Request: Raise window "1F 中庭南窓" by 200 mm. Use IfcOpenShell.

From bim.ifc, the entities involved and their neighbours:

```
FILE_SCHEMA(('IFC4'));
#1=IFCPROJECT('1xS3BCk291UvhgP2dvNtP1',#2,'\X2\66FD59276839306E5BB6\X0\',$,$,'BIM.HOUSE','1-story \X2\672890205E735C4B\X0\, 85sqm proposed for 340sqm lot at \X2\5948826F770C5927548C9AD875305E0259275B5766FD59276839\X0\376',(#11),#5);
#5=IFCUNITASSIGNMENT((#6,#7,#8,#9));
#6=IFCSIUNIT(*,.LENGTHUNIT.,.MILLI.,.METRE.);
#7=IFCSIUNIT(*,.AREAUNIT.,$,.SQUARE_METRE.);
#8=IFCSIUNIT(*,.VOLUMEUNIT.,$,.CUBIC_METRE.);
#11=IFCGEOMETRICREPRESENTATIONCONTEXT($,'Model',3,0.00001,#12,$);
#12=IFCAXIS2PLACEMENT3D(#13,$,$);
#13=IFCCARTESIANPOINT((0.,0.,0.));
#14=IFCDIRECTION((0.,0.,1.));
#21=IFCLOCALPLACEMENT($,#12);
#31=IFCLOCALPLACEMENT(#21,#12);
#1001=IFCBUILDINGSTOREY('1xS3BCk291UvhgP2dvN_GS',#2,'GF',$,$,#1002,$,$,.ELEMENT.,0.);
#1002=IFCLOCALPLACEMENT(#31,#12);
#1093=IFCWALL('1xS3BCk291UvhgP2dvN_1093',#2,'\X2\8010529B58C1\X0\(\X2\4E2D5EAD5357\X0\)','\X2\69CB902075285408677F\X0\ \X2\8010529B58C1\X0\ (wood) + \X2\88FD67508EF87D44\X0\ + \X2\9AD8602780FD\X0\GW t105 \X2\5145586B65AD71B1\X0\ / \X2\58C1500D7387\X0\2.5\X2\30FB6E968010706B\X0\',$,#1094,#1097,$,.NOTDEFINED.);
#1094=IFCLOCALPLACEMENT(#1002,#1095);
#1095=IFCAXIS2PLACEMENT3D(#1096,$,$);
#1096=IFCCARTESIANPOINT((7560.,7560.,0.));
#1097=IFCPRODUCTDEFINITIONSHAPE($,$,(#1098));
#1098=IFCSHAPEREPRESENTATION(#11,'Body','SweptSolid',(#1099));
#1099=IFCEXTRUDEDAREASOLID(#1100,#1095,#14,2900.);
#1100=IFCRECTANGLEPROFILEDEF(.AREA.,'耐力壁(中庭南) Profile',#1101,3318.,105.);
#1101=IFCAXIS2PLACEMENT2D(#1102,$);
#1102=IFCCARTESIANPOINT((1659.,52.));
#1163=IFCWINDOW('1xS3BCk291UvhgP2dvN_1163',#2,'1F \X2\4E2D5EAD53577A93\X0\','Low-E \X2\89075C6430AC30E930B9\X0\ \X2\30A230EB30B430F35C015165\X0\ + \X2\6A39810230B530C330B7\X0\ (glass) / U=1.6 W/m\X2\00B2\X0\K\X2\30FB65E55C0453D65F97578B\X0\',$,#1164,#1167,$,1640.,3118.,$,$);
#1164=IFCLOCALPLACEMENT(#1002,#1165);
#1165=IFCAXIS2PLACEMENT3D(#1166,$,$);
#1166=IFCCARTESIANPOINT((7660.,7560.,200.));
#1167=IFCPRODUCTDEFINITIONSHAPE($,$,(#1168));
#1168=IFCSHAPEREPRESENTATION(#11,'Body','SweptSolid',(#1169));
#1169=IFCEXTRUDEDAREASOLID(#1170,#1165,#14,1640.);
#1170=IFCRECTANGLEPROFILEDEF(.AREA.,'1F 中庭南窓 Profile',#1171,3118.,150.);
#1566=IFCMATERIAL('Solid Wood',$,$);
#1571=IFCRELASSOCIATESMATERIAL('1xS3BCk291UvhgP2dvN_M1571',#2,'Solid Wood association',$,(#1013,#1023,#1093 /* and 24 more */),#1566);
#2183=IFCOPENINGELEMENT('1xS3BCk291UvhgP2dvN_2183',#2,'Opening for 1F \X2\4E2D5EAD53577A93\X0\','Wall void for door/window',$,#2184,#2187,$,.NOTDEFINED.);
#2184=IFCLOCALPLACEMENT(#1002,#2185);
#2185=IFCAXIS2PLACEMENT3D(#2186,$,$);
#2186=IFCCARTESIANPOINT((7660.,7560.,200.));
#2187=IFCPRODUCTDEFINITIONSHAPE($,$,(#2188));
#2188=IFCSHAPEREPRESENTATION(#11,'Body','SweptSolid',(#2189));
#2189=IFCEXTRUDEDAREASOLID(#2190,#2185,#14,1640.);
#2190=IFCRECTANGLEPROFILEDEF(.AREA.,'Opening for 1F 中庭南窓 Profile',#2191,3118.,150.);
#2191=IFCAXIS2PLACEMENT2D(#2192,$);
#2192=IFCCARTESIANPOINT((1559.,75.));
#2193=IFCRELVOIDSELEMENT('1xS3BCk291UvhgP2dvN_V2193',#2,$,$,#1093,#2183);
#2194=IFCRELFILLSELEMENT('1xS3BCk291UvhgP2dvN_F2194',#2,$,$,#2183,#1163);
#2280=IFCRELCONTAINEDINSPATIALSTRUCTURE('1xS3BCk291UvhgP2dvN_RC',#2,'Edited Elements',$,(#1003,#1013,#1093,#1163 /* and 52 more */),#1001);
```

```python
import numpy as np
import ifcopenshell
import ifcopenshell.api.geometry
import ifcopenshell.util.placement
import ifcopenshell.util.unit

model = ifcopenshell.open("bim.ifc")
unit_scale = ifcopenshell.util.unit.calculate_unit_scale(model)

window = model.by_id(1163)
opening = window.FillsVoids[0].RelatingOpeningElement
dz = 0.2 / unit_scale

shift = np.array([0.0, 0.0, dz])
# The window is not placed relative to its opening, so move both.
for product in (opening, window):
    matrix = ifcopenshell.util.placement.get_local_placement(product.ObjectPlacement)
    matrix[:3, 3] += shift
    ifcopenshell.api.geometry.edit_object_placement(model, product=product, matrix=matrix, is_si=False)

print(f"moved by {dz * unit_scale:+.3f} m")

model.write("bim-out.ifc")
```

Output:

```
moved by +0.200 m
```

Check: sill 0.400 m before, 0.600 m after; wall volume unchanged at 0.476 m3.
